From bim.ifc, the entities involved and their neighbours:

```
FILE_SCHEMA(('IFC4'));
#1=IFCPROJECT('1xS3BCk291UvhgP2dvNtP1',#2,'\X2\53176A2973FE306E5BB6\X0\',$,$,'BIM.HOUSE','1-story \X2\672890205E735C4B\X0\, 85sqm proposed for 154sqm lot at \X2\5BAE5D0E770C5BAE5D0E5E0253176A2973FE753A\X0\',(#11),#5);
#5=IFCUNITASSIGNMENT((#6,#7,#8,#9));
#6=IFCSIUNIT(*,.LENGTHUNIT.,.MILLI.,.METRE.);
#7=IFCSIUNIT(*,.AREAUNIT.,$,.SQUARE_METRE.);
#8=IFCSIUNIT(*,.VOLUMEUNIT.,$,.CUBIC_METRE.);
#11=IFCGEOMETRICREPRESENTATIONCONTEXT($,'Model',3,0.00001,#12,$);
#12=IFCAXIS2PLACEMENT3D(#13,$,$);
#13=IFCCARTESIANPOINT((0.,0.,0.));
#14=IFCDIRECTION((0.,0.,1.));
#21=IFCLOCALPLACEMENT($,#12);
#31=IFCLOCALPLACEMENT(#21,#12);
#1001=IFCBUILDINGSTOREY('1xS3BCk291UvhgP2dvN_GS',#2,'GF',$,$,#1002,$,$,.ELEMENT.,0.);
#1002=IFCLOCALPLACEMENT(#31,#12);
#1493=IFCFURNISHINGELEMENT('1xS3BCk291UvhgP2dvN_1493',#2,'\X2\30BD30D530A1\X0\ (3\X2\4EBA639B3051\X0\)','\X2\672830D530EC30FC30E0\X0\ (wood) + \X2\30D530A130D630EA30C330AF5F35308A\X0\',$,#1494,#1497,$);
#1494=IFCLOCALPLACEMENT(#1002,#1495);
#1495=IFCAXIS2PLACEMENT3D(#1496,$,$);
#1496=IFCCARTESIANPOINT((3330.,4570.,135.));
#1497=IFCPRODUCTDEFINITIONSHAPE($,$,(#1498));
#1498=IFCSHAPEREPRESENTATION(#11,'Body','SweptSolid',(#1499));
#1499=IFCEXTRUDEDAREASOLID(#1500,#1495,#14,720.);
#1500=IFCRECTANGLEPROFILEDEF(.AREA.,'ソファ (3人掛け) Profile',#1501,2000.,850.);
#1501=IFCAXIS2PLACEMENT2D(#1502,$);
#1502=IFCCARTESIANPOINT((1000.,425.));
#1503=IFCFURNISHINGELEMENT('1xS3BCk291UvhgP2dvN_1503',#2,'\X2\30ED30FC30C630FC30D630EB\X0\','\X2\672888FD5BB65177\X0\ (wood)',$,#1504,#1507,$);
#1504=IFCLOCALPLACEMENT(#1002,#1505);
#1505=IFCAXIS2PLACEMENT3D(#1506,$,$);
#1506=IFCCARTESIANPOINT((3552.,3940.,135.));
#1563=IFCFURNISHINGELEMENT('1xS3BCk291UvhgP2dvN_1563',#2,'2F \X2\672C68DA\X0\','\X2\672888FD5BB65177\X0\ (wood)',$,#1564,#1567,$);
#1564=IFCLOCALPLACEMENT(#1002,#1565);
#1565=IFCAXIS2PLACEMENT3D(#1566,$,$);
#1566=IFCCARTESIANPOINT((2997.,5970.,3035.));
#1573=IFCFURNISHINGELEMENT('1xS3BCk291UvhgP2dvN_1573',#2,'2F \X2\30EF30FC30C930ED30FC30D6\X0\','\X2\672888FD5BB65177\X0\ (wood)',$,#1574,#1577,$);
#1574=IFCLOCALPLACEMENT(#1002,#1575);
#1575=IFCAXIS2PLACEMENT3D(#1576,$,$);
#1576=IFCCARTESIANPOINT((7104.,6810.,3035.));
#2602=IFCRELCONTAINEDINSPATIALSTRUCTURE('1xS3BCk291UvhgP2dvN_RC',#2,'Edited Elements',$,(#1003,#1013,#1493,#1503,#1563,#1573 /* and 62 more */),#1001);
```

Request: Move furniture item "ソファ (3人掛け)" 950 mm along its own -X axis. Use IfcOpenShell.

```python
import ifcopenshell
import ifcopenshell.api.geometry
import ifcopenshell.util.placement
import ifcopenshell.util.unit

model = ifcopenshell.open("bim.ifc")
unit_scale = ifcopenshell.util.unit.calculate_unit_scale(model)

item = model.by_guid("1xS3BCk291UvhgP2dvN_1493")
matrix = ifcopenshell.util.placement.get_local_placement(item.ObjectPlacement)
matrix[:3, 3] -= matrix[:3, 0] * 0.95 / unit_scale
ifcopenshell.api.geometry.edit_object_placement(model, product=item, matrix=matrix, is_si=False)

print(ifcopenshell.util.placement.get_local_placement(item.ObjectPlacement).round(3) + 0.0)

model.write("bim_rev.ifc")
```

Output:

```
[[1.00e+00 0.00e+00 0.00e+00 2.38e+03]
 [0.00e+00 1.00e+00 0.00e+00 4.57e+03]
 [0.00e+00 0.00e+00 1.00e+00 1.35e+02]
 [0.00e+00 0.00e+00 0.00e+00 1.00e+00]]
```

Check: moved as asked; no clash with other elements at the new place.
